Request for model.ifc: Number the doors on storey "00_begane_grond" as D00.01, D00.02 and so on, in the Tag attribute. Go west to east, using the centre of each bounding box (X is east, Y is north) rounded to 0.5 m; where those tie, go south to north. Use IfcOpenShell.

First a look at what the model holds.

```python
import ifcopenshell
import ifcopenshell.util.element
import ifcopenshell.util.placement

model = ifcopenshell.open("model.ifc")
print(model.schema)
storey = next(s for s in model.by_type("IfcBuildingStorey") if s.Name == "00_begane_grond")
doors = [e for e in ifcopenshell.util.element.get_decomposition(storey) if e.is_a("IfcDoor")]
for e in sorted(doors, key=lambda e: e.id()):
    origin = ifcopenshell.util.placement.get_local_placement(e.ObjectPlacement)[:3, 3]
    print(e.id(), e.Tag, e.Name, origin.round(2) + 0.0, sep=" | ")
```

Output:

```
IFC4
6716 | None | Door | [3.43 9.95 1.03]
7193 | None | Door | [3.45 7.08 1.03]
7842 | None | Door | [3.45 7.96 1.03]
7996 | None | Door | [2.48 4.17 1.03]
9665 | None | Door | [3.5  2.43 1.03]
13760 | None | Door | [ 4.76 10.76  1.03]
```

```python
import ifcopenshell
import ifcopenshell.geom
import ifcopenshell.util.element
import ifcopenshell.util.shape

model = ifcopenshell.open("model.ifc")
settings = ifcopenshell.geom.settings()
settings.set("use-world-coords", True)


def centre(element):
    shape = ifcopenshell.geom.create_shape(settings, element)
    return ifcopenshell.util.shape.get_bbox_centroid(shape.geometry)


storey = next(s for s in model.by_type("IfcBuildingStorey") if s.Name == "00_begane_grond")
doors = [e for e in ifcopenshell.util.element.get_decomposition(storey) if e.is_a("IfcDoor")]

# Insertion points can sit at a corner or the storey origin, so sort by the geometry (in metres).
centres = {e: centre(e) for e in doors}
doors.sort(key=lambda e: (round(centres[e][0] / 0.5), centres[e][1]))

for i, e in enumerate(doors, start=1):
    number = f"D00.{i:02d}"
    e.Tag = number
    print(e.id(), number)

model.write("model_edited.ifc")
```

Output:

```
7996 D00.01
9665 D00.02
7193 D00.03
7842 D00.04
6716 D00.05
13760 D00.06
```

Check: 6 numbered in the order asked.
